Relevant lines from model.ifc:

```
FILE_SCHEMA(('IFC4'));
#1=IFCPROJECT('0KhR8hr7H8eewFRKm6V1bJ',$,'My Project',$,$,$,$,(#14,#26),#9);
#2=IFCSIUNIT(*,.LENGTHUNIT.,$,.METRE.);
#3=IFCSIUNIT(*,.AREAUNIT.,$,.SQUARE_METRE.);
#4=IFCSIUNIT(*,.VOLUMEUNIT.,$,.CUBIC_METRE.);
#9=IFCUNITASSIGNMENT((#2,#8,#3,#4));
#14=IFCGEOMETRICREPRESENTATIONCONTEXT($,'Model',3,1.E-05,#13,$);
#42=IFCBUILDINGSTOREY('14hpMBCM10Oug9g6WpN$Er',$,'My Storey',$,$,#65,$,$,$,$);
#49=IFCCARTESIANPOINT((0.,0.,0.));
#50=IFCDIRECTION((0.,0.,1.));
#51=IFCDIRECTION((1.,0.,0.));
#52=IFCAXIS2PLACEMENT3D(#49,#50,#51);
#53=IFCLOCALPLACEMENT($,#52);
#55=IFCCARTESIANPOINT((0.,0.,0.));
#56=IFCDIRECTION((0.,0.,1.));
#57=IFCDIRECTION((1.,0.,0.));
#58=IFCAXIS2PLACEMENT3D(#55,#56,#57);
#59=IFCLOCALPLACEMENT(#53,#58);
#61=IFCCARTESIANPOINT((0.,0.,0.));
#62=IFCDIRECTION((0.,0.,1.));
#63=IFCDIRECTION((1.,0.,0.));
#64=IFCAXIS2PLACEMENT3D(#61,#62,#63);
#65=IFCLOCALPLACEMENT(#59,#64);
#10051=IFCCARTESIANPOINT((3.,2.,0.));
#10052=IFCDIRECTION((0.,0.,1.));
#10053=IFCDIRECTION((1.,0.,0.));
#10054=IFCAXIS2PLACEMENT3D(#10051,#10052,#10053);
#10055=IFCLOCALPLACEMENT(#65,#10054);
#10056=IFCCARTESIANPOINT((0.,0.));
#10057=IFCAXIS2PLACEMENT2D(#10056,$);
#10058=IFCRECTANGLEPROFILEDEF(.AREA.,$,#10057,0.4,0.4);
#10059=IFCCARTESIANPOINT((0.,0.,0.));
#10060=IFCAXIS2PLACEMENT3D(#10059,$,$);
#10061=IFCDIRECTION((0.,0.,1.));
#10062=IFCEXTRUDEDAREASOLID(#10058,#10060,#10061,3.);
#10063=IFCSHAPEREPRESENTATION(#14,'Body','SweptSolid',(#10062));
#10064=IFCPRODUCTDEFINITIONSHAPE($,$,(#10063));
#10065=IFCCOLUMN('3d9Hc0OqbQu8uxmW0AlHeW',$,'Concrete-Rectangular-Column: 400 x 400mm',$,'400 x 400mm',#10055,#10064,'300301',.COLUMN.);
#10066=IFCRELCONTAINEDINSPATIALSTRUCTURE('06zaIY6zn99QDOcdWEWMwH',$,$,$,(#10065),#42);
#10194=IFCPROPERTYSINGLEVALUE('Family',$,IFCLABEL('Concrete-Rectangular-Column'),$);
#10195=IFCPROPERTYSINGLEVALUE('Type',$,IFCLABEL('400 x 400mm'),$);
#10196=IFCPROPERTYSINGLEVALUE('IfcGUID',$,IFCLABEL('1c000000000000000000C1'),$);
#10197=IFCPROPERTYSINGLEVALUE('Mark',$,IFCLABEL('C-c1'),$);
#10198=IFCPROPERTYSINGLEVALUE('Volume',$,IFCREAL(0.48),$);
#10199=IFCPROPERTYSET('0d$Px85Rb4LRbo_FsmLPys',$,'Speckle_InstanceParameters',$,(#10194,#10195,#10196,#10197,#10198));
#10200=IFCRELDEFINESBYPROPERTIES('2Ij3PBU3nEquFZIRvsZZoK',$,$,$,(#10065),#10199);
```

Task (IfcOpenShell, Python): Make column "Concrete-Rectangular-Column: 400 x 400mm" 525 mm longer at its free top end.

```python
import ifcopenshell
import ifcopenshell.api.pset
import ifcopenshell.util.element
import ifcopenshell.util.unit

model = ifcopenshell.open("model.ifc")
unit_scale = ifcopenshell.util.unit.calculate_unit_scale(model)

member = model.by_guid("3d9Hc0OqbQu8uxmW0AlHeW")
change = 0.525 / unit_scale

# The extrusion runs towards the end named, so only its depth changes.
body = next(r for r in member.Representation.Representations if r.RepresentationIdentifier == "Body")
solid = body.Items[0]
old_length = solid.Depth
solid.Depth += change

# Update the stored length and volume.
pset = model.by_id(ifcopenshell.util.element.get_pset(member, "Speckle_InstanceParameters", should_inherit=False)["id"])
ifcopenshell.api.pset.edit_pset(model, pset=pset, properties={
    "Volume": model.create_entity("IfcReal", ifcopenshell.util.element.get_pset(member, "Speckle_InstanceParameters", "Volume") * solid.Depth / old_length),
})

print(f"length {old_length:g} -> {solid.Depth:g}")

model.write("model-out.ifc")
```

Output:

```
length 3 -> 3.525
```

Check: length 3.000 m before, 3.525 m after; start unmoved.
